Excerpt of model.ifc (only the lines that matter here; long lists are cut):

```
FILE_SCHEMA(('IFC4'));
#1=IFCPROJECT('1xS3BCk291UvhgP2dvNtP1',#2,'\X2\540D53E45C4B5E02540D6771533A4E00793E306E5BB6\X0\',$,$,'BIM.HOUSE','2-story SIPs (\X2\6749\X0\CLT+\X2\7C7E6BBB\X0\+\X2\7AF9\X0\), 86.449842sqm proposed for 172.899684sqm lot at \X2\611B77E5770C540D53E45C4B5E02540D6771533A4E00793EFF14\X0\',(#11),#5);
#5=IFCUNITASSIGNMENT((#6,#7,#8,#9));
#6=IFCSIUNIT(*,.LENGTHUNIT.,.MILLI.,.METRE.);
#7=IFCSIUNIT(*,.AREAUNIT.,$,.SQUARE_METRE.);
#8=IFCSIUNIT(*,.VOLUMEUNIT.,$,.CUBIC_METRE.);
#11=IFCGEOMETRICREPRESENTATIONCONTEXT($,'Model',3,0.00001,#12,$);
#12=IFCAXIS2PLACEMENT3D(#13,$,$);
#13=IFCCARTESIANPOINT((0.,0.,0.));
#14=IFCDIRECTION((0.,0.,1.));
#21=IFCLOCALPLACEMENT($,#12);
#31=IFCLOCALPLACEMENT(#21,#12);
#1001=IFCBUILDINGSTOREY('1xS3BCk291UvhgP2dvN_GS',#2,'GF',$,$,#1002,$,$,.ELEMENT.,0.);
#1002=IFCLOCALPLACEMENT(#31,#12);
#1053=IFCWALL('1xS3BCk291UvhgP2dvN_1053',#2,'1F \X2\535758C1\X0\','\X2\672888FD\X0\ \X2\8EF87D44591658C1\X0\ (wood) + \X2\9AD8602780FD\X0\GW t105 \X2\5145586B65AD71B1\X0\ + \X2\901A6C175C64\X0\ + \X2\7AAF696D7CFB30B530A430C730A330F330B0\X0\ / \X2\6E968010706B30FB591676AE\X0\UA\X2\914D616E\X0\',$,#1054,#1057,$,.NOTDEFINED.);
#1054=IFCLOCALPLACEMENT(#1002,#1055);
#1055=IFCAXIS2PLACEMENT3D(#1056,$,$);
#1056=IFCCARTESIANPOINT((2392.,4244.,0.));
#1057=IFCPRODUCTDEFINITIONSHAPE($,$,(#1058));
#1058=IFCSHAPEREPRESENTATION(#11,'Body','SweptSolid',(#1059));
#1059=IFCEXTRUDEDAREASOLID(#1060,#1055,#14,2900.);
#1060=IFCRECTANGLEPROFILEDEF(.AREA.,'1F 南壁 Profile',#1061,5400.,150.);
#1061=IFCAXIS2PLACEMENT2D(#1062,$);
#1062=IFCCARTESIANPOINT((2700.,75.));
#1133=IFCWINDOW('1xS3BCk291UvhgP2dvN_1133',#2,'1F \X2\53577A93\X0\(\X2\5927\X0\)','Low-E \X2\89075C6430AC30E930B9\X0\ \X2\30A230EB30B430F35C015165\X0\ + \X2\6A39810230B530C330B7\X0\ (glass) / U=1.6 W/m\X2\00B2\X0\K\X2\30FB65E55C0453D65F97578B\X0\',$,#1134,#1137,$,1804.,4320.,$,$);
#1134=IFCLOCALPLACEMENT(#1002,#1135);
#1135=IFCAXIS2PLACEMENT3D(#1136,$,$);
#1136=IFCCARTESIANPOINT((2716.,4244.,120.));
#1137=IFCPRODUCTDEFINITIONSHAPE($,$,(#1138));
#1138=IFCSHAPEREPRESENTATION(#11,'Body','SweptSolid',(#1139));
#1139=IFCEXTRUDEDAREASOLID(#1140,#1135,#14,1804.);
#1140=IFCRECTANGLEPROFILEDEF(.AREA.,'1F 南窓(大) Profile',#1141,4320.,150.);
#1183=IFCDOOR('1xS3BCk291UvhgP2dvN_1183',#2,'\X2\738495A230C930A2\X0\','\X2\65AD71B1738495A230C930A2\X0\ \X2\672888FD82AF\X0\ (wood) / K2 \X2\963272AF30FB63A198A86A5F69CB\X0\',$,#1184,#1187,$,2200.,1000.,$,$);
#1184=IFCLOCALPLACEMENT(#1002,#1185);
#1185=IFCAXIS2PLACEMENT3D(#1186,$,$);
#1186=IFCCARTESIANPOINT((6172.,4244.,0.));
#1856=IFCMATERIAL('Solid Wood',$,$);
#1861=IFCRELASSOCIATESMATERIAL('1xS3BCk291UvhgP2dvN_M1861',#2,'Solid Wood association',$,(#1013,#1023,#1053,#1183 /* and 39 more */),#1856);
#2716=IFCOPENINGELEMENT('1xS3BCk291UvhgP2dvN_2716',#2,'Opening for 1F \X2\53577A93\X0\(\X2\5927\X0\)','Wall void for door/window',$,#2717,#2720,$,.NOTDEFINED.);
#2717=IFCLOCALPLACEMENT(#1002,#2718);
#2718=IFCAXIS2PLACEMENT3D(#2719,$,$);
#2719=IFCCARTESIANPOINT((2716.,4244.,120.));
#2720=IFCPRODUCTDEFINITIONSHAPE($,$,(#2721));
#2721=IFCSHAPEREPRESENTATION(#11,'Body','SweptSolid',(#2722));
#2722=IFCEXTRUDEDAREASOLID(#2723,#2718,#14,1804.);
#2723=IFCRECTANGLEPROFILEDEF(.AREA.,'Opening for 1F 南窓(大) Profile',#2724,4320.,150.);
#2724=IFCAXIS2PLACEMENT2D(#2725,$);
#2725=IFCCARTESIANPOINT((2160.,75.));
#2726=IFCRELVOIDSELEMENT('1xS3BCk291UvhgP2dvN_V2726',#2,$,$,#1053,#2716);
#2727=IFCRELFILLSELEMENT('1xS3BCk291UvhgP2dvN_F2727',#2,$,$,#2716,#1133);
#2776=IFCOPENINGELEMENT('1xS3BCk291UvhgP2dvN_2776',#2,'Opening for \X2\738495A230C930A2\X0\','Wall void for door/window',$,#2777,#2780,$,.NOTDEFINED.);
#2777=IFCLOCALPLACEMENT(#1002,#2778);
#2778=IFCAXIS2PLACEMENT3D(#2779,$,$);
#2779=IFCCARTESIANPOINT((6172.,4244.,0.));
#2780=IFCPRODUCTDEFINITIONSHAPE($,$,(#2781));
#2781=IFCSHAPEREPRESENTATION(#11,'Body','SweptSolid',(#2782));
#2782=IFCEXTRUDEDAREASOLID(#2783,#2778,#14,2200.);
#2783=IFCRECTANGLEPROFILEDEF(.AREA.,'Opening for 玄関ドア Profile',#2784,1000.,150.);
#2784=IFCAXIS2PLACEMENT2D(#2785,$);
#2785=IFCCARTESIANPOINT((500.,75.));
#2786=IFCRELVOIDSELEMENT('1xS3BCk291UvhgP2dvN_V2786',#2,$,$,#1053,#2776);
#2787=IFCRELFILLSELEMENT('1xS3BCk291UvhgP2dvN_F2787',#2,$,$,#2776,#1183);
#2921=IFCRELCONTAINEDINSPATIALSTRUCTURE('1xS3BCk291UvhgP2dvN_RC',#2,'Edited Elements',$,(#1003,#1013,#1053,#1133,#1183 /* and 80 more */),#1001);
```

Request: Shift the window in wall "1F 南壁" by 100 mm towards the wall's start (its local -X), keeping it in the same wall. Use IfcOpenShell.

```python
import ifcopenshell
import ifcopenshell.api.geometry
import ifcopenshell.util.placement
import ifcopenshell.util.unit

model = ifcopenshell.open("model.ifc")
unit_scale = ifcopenshell.util.unit.calculate_unit_scale(model)

window = model.by_guid("1xS3BCk291UvhgP2dvN_1133")
opening = window.FillsVoids[0].RelatingOpeningElement
wall = opening.VoidsElements[0].RelatingBuildingElement

wall_matrix = ifcopenshell.util.placement.get_local_placement(wall.ObjectPlacement)
shift = wall_matrix[:3, 0] * -0.1 / unit_scale
before = ifcopenshell.util.placement.get_local_placement(window.ObjectPlacement)[:3, 3].copy()

# The window is not placed relative to its opening, so move both.
for product in (opening, window):
    matrix = ifcopenshell.util.placement.get_local_placement(product.ObjectPlacement)
    matrix[:3, 3] += shift
    ifcopenshell.api.geometry.edit_object_placement(model, product=product, matrix=matrix, is_si=False)

after = ifcopenshell.util.placement.get_local_placement(window.ObjectPlacement)[:3, 3]
print("window moved by", (after - before).round(3) + 0.0)

model.write("model_updated.ifc")
```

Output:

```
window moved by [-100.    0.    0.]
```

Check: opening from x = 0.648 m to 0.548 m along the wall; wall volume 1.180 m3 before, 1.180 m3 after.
